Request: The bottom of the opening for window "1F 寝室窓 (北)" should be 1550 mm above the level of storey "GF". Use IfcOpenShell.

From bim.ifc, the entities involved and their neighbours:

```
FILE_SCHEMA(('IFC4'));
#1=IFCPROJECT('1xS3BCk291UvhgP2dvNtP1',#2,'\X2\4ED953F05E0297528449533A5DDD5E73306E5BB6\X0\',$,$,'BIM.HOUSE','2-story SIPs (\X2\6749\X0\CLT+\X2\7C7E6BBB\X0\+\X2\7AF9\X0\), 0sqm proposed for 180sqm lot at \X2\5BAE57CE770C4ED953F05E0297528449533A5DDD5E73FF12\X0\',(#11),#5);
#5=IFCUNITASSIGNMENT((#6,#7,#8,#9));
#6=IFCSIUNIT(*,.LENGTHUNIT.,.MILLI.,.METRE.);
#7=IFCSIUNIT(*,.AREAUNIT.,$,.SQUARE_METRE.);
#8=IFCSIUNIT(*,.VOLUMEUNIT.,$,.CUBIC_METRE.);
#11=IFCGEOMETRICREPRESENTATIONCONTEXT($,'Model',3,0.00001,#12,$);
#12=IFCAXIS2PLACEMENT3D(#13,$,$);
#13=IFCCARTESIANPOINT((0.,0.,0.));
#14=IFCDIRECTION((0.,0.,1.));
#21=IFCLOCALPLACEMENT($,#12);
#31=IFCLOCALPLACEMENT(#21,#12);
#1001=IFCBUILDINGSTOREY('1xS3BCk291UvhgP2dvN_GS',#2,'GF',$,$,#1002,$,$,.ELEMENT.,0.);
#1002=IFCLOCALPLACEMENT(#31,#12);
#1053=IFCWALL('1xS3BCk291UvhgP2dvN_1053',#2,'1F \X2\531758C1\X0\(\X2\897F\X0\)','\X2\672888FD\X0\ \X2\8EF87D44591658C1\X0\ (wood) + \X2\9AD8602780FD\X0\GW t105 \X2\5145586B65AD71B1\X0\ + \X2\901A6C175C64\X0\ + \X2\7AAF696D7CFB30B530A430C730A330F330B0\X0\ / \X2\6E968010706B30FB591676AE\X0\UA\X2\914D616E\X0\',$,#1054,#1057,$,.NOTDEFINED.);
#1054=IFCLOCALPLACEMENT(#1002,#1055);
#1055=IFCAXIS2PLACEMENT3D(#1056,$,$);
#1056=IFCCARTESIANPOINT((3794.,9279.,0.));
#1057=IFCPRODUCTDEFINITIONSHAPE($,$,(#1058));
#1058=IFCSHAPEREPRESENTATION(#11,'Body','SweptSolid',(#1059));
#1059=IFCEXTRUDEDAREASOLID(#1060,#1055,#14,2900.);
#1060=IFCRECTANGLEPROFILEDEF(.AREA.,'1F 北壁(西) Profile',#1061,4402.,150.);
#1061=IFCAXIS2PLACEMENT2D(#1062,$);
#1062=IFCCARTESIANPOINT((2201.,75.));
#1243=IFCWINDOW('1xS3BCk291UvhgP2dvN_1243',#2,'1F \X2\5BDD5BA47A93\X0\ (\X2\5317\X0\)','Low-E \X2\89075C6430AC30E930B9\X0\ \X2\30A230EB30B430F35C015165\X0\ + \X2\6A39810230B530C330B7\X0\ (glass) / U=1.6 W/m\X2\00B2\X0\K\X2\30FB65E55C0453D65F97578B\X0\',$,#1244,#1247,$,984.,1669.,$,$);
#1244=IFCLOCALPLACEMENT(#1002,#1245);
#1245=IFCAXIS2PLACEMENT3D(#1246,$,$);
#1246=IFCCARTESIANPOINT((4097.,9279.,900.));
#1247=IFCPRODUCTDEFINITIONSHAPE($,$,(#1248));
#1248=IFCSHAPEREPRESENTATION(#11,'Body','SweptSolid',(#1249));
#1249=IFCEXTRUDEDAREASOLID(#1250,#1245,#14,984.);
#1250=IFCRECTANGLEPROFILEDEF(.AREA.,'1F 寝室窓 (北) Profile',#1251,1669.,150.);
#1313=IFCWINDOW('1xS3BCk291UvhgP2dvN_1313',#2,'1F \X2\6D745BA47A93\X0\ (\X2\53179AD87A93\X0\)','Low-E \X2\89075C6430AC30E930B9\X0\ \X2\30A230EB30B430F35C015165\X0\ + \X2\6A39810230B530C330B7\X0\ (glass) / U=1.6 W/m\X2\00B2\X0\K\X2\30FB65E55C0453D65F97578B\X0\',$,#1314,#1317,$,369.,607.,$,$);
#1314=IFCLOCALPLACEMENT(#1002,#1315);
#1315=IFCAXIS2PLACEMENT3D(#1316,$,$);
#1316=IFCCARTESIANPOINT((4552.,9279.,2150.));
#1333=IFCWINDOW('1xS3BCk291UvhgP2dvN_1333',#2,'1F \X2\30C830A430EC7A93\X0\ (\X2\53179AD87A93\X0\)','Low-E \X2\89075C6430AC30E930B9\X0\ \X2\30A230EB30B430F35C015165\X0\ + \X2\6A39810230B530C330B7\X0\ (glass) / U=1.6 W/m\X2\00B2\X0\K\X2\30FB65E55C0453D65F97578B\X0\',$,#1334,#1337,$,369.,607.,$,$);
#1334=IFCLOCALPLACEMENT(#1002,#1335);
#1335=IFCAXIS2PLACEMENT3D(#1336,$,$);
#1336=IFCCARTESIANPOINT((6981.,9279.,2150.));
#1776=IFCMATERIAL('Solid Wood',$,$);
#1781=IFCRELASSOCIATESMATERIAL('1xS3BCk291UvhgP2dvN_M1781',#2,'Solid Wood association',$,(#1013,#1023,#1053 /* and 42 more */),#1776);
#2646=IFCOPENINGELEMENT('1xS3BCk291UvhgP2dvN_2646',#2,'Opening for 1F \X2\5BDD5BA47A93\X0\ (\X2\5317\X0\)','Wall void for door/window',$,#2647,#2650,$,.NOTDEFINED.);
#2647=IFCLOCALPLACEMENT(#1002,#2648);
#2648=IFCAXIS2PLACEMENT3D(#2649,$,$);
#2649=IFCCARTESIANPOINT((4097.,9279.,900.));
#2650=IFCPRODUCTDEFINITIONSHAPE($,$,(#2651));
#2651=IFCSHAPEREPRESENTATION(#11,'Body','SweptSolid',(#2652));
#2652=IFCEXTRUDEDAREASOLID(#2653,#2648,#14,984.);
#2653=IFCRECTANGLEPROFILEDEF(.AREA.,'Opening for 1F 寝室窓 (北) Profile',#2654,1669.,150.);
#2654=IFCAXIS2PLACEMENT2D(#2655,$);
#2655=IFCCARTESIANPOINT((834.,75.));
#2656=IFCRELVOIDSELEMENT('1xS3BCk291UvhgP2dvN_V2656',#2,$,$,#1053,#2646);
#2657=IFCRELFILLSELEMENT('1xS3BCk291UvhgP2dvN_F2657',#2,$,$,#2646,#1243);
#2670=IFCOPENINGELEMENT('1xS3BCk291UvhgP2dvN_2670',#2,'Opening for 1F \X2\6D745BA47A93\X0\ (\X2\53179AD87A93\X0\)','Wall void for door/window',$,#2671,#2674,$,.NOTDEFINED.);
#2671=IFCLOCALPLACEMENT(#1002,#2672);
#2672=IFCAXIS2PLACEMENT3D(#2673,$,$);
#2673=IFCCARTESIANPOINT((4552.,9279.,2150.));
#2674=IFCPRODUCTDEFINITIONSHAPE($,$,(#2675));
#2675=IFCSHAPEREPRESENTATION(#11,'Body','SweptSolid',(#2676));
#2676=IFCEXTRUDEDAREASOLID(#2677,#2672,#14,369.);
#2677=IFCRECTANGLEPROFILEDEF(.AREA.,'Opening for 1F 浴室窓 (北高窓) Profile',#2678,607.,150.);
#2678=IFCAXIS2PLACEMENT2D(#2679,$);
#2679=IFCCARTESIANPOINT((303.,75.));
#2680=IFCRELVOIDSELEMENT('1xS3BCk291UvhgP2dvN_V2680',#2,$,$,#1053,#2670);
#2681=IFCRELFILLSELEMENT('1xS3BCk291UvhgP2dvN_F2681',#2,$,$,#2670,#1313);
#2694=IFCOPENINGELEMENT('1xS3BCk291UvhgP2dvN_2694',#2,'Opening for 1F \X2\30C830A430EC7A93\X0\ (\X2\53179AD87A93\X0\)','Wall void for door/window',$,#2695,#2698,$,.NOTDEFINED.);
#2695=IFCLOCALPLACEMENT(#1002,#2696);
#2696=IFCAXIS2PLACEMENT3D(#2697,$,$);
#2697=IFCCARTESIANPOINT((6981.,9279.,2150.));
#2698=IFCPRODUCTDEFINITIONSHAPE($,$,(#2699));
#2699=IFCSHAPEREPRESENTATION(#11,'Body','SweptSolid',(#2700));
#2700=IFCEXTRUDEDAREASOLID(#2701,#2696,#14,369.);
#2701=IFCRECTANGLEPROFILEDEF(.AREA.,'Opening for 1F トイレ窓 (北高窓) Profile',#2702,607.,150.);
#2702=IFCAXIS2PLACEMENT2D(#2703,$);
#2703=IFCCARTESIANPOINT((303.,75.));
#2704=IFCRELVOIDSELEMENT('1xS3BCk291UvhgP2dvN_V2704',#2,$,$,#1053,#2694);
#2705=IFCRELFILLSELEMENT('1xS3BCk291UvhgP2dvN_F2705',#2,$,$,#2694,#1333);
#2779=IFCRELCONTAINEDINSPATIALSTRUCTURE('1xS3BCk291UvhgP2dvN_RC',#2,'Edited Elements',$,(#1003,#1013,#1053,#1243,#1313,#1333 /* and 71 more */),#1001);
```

```python
import numpy as np
import ifcopenshell
import ifcopenshell.api.geometry
import ifcopenshell.geom
import ifcopenshell.util.element
import ifcopenshell.util.placement
import ifcopenshell.util.shape
import ifcopenshell.util.unit

model = ifcopenshell.open("bim.ifc")
unit_scale = ifcopenshell.util.unit.calculate_unit_scale(model)

window = model.by_guid("1xS3BCk291UvhgP2dvN_1243")
opening = window.FillsVoids[0].RelatingOpeningElement
storey = ifcopenshell.util.element.get_container(window, ifc_class="IfcBuildingStorey")
level = ifcopenshell.util.placement.get_local_placement(storey.ObjectPlacement)[2, 3]

# The opening's origin need not be at the sill, so measure its lowest point.
shape = ifcopenshell.geom.create_shape(ifcopenshell.geom.settings(), opening)
bottom = ifcopenshell.util.shape.get_shape_bottom_elevation(shape, shape.geometry) / unit_scale
dz = level + 1550.0 - bottom

shift = np.array([0.0, 0.0, dz])
# The window is not placed relative to its opening, so move both.
for product in (opening, window):
    matrix = ifcopenshell.util.placement.get_local_placement(product.ObjectPlacement)
    matrix[:3, 3] += shift
    ifcopenshell.api.geometry.edit_object_placement(model, product=product, matrix=matrix, is_si=False)

print(f"moved by {dz * unit_scale:+.3f} m")

model.write("bim_updated.ifc")
```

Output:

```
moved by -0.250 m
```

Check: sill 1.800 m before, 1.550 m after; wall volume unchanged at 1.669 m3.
